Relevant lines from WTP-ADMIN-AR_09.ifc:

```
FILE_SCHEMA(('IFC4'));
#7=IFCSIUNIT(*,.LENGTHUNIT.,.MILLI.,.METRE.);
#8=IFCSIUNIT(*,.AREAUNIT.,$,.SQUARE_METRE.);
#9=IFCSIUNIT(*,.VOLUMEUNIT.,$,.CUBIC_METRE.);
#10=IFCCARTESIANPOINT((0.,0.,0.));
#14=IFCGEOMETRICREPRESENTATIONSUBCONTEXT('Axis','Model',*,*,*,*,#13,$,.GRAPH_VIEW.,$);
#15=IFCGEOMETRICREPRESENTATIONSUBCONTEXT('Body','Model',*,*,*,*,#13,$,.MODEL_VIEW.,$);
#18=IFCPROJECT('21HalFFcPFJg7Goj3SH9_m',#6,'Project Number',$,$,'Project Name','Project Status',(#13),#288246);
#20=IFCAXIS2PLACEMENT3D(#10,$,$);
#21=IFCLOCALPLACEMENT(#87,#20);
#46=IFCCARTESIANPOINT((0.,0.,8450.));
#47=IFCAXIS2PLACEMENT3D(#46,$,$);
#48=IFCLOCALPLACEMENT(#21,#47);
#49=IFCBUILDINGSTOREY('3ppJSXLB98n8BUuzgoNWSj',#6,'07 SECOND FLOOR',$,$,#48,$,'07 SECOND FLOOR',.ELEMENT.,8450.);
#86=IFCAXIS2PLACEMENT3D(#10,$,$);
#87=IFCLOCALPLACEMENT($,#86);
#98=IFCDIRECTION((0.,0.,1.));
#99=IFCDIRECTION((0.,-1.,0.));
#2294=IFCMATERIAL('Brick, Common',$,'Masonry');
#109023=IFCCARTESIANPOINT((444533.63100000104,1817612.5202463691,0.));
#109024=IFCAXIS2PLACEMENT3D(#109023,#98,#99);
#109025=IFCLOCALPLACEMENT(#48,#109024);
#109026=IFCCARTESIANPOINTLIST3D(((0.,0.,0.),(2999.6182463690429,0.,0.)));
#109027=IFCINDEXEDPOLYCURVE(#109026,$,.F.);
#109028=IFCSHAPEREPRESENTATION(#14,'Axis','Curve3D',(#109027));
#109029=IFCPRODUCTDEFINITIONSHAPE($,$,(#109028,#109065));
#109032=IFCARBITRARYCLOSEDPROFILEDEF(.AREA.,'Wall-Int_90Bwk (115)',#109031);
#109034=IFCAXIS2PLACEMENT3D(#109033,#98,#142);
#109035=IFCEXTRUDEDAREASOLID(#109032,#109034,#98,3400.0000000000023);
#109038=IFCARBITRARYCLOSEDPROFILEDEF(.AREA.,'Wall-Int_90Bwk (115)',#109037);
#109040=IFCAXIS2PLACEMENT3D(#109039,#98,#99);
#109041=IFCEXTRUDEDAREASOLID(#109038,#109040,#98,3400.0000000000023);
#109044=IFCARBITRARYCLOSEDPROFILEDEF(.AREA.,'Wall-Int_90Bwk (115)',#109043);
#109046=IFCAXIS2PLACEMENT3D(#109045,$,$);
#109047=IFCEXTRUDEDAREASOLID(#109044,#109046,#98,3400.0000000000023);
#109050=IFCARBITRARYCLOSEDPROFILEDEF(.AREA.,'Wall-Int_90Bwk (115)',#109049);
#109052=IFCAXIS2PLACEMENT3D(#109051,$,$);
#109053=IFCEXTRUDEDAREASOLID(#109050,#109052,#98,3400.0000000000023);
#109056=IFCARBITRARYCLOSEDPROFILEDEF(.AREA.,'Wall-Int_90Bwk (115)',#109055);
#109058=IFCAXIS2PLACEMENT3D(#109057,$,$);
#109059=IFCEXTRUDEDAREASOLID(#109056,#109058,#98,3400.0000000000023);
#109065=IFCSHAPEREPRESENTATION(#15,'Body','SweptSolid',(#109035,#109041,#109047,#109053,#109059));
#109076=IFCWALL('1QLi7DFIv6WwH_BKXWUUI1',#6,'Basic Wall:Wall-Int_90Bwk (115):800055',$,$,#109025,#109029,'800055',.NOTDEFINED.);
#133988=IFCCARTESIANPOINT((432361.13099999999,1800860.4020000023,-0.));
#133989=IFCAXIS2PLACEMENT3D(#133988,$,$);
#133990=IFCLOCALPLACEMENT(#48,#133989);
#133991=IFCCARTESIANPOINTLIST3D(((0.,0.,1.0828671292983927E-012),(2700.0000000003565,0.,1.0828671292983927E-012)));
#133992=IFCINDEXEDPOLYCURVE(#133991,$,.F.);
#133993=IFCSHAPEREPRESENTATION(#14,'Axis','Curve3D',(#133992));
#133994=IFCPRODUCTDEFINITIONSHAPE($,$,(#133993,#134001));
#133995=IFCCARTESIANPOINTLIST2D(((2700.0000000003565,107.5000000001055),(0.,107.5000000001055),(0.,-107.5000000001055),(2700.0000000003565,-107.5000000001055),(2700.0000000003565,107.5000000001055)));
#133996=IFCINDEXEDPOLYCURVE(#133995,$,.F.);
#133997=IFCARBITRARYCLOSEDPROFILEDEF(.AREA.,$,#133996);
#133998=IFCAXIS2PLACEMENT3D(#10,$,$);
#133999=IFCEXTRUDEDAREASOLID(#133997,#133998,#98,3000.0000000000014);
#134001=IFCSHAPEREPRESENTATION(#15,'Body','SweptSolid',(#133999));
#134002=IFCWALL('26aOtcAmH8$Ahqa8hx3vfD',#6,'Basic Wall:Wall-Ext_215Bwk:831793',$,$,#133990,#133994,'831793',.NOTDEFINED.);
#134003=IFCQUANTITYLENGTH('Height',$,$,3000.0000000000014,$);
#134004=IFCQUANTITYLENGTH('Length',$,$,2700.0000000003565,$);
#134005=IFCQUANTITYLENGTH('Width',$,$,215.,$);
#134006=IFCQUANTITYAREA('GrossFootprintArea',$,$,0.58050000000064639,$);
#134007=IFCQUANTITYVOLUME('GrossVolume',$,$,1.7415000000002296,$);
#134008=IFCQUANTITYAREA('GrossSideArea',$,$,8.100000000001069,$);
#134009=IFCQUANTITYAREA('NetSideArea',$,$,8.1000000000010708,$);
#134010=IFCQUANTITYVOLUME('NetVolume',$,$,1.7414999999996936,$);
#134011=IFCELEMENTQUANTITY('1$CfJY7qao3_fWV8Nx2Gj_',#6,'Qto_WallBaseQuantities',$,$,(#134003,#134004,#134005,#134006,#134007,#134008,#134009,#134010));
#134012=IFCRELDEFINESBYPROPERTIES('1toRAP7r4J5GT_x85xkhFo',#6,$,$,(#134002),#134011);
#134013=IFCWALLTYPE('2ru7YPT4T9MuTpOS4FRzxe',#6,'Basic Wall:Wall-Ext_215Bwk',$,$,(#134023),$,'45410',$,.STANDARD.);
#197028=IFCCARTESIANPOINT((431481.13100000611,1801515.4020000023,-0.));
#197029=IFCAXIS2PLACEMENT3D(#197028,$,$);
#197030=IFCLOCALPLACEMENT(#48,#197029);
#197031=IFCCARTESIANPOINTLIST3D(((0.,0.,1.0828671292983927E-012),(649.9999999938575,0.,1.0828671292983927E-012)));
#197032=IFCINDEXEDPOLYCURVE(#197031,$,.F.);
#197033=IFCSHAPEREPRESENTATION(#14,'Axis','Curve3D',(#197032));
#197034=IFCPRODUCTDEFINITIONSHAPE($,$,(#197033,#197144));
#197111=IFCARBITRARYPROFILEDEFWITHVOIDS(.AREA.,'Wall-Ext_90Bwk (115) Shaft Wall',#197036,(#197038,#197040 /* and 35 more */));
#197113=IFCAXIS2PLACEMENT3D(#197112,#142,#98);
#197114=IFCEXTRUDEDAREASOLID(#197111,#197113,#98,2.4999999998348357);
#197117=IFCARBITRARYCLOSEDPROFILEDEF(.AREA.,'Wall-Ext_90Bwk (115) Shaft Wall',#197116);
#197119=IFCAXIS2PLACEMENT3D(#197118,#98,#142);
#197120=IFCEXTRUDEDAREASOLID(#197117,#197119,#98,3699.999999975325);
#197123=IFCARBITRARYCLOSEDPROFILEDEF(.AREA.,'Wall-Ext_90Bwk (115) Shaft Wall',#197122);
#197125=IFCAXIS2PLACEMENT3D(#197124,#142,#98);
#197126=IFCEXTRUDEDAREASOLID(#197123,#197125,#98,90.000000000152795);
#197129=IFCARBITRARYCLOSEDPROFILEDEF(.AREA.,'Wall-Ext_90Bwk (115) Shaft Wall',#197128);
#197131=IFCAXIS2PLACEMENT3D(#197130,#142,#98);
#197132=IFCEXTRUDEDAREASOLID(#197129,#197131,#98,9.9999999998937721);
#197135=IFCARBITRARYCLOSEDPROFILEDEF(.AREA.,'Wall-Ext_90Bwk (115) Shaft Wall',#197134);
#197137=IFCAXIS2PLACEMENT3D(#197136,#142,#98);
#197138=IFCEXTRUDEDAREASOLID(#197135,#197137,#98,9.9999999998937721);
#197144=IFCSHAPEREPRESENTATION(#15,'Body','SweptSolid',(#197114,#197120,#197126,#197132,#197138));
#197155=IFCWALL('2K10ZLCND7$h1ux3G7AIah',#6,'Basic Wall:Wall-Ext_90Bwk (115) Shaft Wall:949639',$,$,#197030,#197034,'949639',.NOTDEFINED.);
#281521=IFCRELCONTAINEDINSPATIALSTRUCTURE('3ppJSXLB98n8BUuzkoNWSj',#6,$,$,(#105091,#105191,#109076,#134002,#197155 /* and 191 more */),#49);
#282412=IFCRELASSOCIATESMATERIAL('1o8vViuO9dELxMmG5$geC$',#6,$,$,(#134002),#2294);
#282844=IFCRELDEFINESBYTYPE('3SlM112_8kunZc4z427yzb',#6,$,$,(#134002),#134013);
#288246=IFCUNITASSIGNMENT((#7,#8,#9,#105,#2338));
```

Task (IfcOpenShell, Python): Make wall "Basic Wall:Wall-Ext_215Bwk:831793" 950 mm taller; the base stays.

```python
import ifcopenshell
import ifcopenshell.api.pset
import ifcopenshell.geom
import ifcopenshell.util.element
import ifcopenshell.util.representation
import ifcopenshell.util.shape
import ifcopenshell.util.unit

model = ifcopenshell.open("WTP-ADMIN-AR_09.ifc")
unit_scale = ifcopenshell.util.unit.calculate_unit_scale(model)
area_scale = ifcopenshell.util.unit.calculate_unit_scale(model, "AREAUNIT")
volume_scale = ifcopenshell.util.unit.calculate_unit_scale(model, "VOLUMEUNIT")
settings = ifcopenshell.geom.settings()


def volume(element):
    """Net volume in cubic metres, openings subtracted."""
    shape = ifcopenshell.geom.create_shape(settings, element)
    return ifcopenshell.util.shape.get_volume(shape.geometry)


wall = model.by_guid("26aOtcAmH8$Ahqa8hx3vfD")
before = volume(wall)

body = ifcopenshell.util.representation.get_representation(wall, "Model", "Body")
solid = body.Items[0]
old_height = solid.Depth
solid.Depth += 0.95 / unit_scale
after = volume(wall)
thickness = 0.215  # wall thickness in metres

# Update the stored height, areas and volumes.
qto = model.by_id(ifcopenshell.util.element.get_pset(wall, "Qto_WallBaseQuantities", should_inherit=False)["id"])
ifcopenshell.api.pset.edit_qto(model, qto=qto, properties={
    "Height": solid.Depth,
    "GrossVolume": ifcopenshell.util.element.get_pset(wall, "Qto_WallBaseQuantities", "GrossVolume") * solid.Depth / old_height,
    "GrossSideArea": ifcopenshell.util.element.get_pset(wall, "Qto_WallBaseQuantities", "GrossSideArea") * solid.Depth / old_height,
    "NetSideArea": after / thickness / area_scale,
    "NetVolume": after / volume_scale,
})

print(f"height {old_height:g} -> {solid.Depth:g}, volume {before:.3f} -> {after:.3f} m3")

model.write("WTP-ADMIN-AR_09-out.ifc")
```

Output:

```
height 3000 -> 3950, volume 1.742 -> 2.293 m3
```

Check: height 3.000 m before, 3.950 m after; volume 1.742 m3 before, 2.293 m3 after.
